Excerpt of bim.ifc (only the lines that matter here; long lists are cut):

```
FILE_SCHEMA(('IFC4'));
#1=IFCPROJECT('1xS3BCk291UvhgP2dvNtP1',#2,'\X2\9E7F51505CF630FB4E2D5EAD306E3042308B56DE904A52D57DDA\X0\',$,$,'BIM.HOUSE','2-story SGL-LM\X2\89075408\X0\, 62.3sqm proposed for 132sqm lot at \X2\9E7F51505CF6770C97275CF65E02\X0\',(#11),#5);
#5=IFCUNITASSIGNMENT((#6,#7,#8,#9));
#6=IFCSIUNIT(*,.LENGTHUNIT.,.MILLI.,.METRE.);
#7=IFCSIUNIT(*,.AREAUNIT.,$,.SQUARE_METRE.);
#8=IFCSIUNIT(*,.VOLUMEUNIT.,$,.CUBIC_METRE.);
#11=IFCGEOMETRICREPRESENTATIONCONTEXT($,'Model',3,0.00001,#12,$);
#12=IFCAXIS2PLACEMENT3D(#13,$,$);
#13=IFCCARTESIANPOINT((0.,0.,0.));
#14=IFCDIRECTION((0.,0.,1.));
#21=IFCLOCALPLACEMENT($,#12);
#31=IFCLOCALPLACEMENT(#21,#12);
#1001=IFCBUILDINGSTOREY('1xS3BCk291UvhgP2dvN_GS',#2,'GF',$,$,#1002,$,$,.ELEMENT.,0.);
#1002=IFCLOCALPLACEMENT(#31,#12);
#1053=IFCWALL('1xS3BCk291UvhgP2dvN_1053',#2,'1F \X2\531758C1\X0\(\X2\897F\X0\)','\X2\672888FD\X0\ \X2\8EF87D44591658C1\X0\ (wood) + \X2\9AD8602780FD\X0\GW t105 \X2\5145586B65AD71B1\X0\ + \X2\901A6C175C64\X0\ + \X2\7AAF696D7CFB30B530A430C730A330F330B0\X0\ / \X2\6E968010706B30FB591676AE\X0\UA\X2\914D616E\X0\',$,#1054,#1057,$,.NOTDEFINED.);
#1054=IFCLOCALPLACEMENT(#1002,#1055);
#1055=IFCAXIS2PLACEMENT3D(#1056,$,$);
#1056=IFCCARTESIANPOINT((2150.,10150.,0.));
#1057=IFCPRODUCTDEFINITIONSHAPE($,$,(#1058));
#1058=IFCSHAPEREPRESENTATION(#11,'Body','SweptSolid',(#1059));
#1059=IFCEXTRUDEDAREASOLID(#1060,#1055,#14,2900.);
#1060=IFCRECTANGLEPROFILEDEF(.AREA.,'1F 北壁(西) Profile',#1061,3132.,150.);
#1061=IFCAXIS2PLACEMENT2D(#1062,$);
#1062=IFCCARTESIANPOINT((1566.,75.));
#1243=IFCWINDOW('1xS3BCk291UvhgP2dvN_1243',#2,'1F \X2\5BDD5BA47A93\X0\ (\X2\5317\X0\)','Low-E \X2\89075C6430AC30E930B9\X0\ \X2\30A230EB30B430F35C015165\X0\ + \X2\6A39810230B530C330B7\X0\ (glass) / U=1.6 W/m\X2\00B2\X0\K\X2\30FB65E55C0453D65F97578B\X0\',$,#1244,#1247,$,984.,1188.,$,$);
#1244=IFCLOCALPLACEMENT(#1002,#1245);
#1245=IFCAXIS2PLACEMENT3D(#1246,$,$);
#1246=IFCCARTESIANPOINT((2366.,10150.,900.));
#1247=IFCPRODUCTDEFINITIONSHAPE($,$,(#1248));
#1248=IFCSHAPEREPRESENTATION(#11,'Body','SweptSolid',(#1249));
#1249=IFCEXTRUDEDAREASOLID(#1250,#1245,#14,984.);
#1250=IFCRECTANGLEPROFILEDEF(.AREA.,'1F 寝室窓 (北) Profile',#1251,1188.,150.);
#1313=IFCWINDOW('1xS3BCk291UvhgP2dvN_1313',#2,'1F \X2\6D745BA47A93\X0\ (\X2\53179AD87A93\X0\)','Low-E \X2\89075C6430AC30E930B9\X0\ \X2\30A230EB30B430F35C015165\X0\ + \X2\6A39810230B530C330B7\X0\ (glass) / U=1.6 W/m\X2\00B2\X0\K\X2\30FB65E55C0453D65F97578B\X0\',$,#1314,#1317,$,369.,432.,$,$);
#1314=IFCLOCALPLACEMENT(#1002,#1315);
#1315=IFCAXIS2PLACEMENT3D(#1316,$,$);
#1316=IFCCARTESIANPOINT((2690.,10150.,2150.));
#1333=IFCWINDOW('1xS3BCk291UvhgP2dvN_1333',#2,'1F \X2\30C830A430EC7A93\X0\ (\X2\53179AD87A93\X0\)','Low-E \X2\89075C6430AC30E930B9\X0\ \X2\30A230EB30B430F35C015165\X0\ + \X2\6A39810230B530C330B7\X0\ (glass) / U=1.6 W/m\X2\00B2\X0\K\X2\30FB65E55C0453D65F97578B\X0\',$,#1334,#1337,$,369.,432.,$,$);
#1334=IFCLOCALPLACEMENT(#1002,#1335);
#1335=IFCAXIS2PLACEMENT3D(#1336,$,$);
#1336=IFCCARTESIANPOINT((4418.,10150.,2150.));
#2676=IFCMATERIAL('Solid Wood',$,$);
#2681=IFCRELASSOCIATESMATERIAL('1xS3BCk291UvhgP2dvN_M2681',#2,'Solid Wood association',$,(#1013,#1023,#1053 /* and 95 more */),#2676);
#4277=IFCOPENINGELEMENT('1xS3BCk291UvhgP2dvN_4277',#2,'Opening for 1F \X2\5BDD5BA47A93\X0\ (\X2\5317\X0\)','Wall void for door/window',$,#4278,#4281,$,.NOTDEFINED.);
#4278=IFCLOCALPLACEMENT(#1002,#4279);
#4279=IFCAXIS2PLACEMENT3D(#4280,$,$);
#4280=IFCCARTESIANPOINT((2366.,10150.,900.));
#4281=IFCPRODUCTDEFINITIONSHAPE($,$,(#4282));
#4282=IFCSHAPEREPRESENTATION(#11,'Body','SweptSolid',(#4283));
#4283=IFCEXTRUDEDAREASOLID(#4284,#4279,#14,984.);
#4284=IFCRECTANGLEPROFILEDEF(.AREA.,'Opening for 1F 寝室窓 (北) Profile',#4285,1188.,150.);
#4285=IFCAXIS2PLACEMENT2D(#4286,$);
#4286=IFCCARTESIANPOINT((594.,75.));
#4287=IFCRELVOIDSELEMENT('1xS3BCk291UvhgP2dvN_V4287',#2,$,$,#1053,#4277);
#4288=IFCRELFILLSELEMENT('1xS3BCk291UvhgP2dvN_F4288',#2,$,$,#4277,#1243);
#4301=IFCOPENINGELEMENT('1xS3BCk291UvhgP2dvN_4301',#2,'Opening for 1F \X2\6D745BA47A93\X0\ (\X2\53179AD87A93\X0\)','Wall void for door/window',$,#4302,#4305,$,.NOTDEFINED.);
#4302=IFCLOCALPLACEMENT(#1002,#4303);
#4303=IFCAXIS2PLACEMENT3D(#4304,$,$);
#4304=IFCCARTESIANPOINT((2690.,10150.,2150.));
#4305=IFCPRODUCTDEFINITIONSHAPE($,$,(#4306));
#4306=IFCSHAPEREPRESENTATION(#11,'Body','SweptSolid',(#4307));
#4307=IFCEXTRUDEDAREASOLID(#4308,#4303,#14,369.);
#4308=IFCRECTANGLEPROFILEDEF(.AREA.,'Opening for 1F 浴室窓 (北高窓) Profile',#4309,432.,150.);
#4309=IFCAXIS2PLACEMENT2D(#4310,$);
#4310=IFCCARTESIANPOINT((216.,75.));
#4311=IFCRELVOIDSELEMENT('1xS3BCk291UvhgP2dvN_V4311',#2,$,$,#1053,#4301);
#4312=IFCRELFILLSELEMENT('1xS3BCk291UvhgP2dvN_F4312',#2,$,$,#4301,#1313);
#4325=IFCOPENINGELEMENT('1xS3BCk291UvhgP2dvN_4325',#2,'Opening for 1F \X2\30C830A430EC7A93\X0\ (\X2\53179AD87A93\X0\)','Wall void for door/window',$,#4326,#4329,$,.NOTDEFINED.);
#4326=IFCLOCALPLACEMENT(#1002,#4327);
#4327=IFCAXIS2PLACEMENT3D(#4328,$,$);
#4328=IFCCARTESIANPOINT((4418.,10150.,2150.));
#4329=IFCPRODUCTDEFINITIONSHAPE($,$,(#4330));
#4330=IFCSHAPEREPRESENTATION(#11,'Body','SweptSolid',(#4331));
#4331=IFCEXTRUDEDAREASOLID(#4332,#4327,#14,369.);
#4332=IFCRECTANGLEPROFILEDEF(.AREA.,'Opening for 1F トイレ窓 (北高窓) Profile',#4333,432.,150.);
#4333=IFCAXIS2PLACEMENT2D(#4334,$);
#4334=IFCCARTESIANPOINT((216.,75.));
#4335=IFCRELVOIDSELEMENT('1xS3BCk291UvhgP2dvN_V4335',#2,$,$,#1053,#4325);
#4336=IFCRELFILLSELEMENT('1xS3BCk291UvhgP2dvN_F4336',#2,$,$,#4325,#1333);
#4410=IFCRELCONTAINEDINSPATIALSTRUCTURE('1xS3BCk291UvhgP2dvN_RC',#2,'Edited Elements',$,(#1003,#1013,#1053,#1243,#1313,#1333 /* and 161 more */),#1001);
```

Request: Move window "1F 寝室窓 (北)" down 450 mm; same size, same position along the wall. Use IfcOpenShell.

```python
import numpy as np
import ifcopenshell
import ifcopenshell.api.geometry
import ifcopenshell.util.placement
import ifcopenshell.util.unit

model = ifcopenshell.open("bim.ifc")
unit_scale = ifcopenshell.util.unit.calculate_unit_scale(model)

window = model.by_guid("1xS3BCk291UvhgP2dvN_1243")
opening = window.FillsVoids[0].RelatingOpeningElement
dz = -450.0

shift = np.array([0.0, 0.0, dz])
# The window is not placed relative to its opening, so move both.
for product in (opening, window):
    matrix = ifcopenshell.util.placement.get_local_placement(product.ObjectPlacement)
    matrix[:3, 3] += shift
    ifcopenshell.api.geometry.edit_object_placement(model, product=product, matrix=matrix, is_si=False)

print(f"moved by {dz * unit_scale:+.3f} m")

model.write("bim_v2.ifc")
```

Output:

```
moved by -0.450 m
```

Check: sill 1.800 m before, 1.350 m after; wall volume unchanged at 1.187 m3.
